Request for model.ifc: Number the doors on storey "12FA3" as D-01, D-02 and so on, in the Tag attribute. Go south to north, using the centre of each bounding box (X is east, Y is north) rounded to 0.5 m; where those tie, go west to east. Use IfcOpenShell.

First a look at what the model holds.

```python
import ifcopenshell
import ifcopenshell.util.element
import ifcopenshell.util.placement

model = ifcopenshell.open("model.ifc")
print(model.schema)
storey = next(s for s in model.by_type("IfcBuildingStorey") if s.Name == "12FA3")
doors = [e for e in ifcopenshell.util.element.get_decomposition(storey) if e.is_a("IfcDoor")]
for e in sorted(doors, key=lambda e: e.id()):
    origin = ifcopenshell.util.placement.get_local_placement(e.ObjectPlacement)[:3, 3]
    print(e.id(), e.Tag, e.Name, origin.round(2) + 0.0, sep=" | ")
```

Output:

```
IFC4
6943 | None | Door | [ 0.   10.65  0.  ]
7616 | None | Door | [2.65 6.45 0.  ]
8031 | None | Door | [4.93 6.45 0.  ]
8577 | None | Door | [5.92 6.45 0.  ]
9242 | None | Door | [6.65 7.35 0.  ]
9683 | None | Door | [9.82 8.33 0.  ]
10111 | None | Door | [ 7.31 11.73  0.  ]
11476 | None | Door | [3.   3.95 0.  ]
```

```python
import ifcopenshell
import ifcopenshell.geom
import ifcopenshell.util.element
import ifcopenshell.util.shape

model = ifcopenshell.open("model.ifc")
settings = ifcopenshell.geom.settings()
settings.set("use-world-coords", True)


def centre(element):
    shape = ifcopenshell.geom.create_shape(settings, element)
    return ifcopenshell.util.shape.get_bbox_centroid(shape.geometry)


storey = next(s for s in model.by_type("IfcBuildingStorey") if s.Name == "12FA3")
doors = [e for e in ifcopenshell.util.element.get_decomposition(storey) if e.is_a("IfcDoor")]

# Insertion points can sit at a corner or the storey origin, so sort by the geometry (in metres).
centres = {e: centre(e) for e in doors}
doors.sort(key=lambda e: (round(centres[e][1] / 0.5), centres[e][0]))

for i, e in enumerate(doors, start=1):
    number = f"D-{i:02d}"
    e.Tag = number
    print(e.id(), number)

model.write("model_updated.ifc")
```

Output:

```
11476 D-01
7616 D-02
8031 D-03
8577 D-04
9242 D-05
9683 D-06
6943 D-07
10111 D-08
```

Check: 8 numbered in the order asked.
